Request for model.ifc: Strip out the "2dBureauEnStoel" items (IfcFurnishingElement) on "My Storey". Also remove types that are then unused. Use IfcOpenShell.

First a look at what the model holds.

```python
import ifcopenshell
import ifcopenshell.util.element

model = ifcopenshell.open("model.ifc")
print(model.schema)
storey = next(s for s in model.by_type("IfcBuildingStorey") if s.Name == "My Storey")
furniture = [e for e in ifcopenshell.util.element.get_decomposition(storey) if e.is_a("IfcFurnishingElement")]
seen = {}
for e in furniture:
    element_type = ifcopenshell.util.element.get_type(e)
    name = element_type.Name if element_type not in (None, e) else None
    seen[name] = seen.get(name, 0) + 1
for name, count in sorted(seen.items(), key=str):
    print(count, "x", name)
```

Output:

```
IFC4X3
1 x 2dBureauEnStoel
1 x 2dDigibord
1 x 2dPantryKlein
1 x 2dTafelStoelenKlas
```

```python
import ifcopenshell
import ifcopenshell.api.root
import ifcopenshell.util.element

model = ifcopenshell.open("model.ifc")

storey = next(s for s in model.by_type("IfcBuildingStorey") if s.Name == "My Storey")
furniture = [e for e in ifcopenshell.util.element.get_decomposition(storey) if e.is_a("IfcFurnishingElement")]
targets = [e for e in furniture if (t := ifcopenshell.util.element.get_type(e)) not in (None, e) and t.Name == "2dBureauEnStoel"]
types = {ifcopenshell.util.element.get_type(e) for e in targets} - {None, *targets}

for e in targets:
    ifcopenshell.api.root.remove_product(model, product=e)
print(len(targets), "removed")

unused = [t for t in types if not ifcopenshell.util.element.get_types(t)]
for t in unused:
    ifcopenshell.api.root.remove_product(model, product=t)
print(len(unused), "unused types removed")

model.write("model_edited.ifc")
```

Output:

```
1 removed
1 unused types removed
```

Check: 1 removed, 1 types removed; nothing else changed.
